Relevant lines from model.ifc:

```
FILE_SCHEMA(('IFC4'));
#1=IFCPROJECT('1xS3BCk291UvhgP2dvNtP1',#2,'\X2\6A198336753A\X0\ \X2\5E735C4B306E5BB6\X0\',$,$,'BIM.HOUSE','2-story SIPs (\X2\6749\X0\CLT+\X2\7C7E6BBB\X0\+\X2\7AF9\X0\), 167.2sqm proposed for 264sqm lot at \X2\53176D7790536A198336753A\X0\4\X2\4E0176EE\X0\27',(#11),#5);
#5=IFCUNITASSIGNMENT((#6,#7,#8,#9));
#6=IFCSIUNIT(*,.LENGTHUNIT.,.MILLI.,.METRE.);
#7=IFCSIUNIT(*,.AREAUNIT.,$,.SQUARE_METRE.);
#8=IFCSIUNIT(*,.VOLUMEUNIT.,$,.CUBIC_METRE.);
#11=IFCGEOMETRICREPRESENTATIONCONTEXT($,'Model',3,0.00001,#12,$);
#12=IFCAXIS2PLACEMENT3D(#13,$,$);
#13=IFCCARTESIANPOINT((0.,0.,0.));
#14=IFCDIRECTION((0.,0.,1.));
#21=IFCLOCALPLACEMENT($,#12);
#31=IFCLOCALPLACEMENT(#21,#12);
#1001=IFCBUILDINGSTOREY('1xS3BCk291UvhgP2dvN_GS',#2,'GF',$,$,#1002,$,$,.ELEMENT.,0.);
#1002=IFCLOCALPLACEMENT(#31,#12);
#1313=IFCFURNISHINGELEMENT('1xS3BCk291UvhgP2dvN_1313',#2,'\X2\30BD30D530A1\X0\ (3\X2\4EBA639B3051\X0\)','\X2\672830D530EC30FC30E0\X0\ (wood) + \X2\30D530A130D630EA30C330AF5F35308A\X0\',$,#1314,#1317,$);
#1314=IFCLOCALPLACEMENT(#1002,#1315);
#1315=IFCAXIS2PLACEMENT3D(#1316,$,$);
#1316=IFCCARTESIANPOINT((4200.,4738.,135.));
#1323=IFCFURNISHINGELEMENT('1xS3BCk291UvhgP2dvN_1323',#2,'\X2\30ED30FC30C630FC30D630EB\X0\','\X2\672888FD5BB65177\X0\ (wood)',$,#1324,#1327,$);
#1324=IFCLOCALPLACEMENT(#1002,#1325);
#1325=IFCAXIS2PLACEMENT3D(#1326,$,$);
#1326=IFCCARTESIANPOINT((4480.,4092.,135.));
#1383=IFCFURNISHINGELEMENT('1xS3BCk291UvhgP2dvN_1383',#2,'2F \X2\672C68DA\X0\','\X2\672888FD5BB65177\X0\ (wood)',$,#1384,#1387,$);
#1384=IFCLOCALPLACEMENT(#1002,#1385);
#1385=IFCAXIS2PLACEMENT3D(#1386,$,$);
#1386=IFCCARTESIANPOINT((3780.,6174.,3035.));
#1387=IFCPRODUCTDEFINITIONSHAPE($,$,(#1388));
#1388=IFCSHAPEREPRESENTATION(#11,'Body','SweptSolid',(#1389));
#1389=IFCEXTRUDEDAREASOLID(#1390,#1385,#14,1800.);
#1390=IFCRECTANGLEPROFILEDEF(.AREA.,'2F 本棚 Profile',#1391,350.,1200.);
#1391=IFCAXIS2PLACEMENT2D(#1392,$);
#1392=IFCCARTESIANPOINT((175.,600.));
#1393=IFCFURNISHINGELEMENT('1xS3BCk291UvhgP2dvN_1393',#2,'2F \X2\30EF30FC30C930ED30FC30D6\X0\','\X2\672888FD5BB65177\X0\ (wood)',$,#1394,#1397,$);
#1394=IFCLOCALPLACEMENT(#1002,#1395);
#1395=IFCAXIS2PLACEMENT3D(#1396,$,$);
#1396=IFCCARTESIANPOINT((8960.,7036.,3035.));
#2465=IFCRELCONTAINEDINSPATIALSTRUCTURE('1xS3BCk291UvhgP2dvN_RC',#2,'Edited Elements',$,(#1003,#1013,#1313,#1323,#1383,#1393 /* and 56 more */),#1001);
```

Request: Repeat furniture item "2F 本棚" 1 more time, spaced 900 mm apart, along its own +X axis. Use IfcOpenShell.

```python
import ifcopenshell
import ifcopenshell.api.geometry
import ifcopenshell.api.root
import ifcopenshell.util.element
import ifcopenshell.util.placement
import ifcopenshell.util.unit

model = ifcopenshell.open("model.ifc")
unit_scale = ifcopenshell.util.unit.calculate_unit_scale(model)


def reuse_history(source, copy):
    """copy_class also copies each property set's owner history, people and application; keep the originals."""
    for rel in copy.IsDefinedBy:
        if rel.is_a("IfcRelDefinesByProperties") and (history := rel.RelatingPropertyDefinition.OwnerHistory):
            rel.RelatingPropertyDefinition.OwnerHistory = source.OwnerHistory
            ifcopenshell.util.element.remove_deep2(model, history)


source = model.by_guid("1xS3BCk291UvhgP2dvN_1383")
base = ifcopenshell.util.placement.get_local_placement(source.ObjectPlacement)
step = base[:3, 0] * 0.9 / unit_scale

for i in range(1, 2):
    copy = ifcopenshell.api.root.copy_class(model, product=source)
    copy.Representation = ifcopenshell.util.element.copy_deep(
        model, source.Representation, exclude=["IfcGeometricRepresentationContext", "IfcRepresentationMap"]
    )
    reuse_history(source, copy)
    matrix = base.copy()
    matrix[:3, 3] += i * step
    print("added at", matrix[:3, 3].round(3) + 0.0)
    ifcopenshell.api.geometry.edit_object_placement(model, product=copy, matrix=matrix, is_si=False)

model.write("model_updated.ifc")
```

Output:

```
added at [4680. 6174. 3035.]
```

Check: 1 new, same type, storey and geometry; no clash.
